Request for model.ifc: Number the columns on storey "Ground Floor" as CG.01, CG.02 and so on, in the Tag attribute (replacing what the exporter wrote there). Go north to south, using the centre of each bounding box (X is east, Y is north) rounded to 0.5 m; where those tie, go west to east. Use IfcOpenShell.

First a look at what the model holds.

```python
import ifcopenshell
import ifcopenshell.util.element
import ifcopenshell.util.placement

model = ifcopenshell.open("model.ifc")
print(model.schema)
storey = next(s for s in model.by_type("IfcBuildingStorey") if s.Name == "Ground Floor")
columns = [e for e in ifcopenshell.util.element.get_decomposition(storey) if e.is_a("IfcColumn")]
for e in sorted(columns, key=lambda e: e.id()):
    origin = ifcopenshell.util.placement.get_local_placement(e.ObjectPlacement)[:3, 3]
    print(e.id(), e.Tag, e.Name, origin.round(2) + 0.0, sep=" | ")
```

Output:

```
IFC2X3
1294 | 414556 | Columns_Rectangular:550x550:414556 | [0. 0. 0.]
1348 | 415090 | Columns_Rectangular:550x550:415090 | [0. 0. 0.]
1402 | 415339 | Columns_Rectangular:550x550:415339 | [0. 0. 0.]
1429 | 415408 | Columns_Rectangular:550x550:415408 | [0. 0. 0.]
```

```python
import ifcopenshell
import ifcopenshell.geom
import ifcopenshell.util.element
import ifcopenshell.util.shape

model = ifcopenshell.open("model.ifc")
settings = ifcopenshell.geom.settings()
settings.set("use-world-coords", True)


def centre(element):
    shape = ifcopenshell.geom.create_shape(settings, element)
    return ifcopenshell.util.shape.get_bbox_centroid(shape.geometry)


storey = next(s for s in model.by_type("IfcBuildingStorey") if s.Name == "Ground Floor")
columns = [e for e in ifcopenshell.util.element.get_decomposition(storey) if e.is_a("IfcColumn")]

# Insertion points can sit at a corner or the storey origin, so sort by the geometry (in metres).
centres = {e: centre(e) for e in columns}
columns.sort(key=lambda e: (-round(centres[e][1] / 0.5), centres[e][0]))

for i, e in enumerate(columns, start=1):
    number = f"CG.{i:02d}"
    e.Tag = number
    print(e.id(), number)

model.write("model-out.ifc")
```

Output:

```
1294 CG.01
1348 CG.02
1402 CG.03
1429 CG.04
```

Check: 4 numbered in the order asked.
